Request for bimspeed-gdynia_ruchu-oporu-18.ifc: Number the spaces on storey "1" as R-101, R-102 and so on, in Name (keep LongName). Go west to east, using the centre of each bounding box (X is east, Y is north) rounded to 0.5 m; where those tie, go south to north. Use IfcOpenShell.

First a look at what the model holds.

```python
import ifcopenshell
import ifcopenshell.util.element
import ifcopenshell.util.placement

model = ifcopenshell.open("bimspeed-gdynia_ruchu-oporu-18.ifc")
print(model.schema)
storey = next(s for s in model.by_type("IfcBuildingStorey") if s.Name == "1")
spaces = [e for e in ifcopenshell.util.element.get_decomposition(storey) if e.is_a("IfcSpace")]
for e in sorted(spaces, key=lambda e: e.id()):
    origin = ifcopenshell.util.placement.get_local_placement(e.ObjectPlacement)[:3, 3]
    print(e.id(), e.Name, e.LongName, origin.round(2) + 0.0, sep=" | ")
```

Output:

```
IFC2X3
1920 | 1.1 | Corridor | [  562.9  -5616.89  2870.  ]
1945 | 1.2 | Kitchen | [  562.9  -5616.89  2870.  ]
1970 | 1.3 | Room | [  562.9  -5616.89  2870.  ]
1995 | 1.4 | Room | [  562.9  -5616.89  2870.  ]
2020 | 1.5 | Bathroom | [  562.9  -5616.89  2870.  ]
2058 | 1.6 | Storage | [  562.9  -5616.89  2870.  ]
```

```python
import ifcopenshell
import ifcopenshell.geom
import ifcopenshell.util.element
import ifcopenshell.util.shape

model = ifcopenshell.open("bimspeed-gdynia_ruchu-oporu-18.ifc")
settings = ifcopenshell.geom.settings()
settings.set("use-world-coords", True)


def centre(element):
    shape = ifcopenshell.geom.create_shape(settings, element)
    return ifcopenshell.util.shape.get_bbox_centroid(shape.geometry)


storey = next(s for s in model.by_type("IfcBuildingStorey") if s.Name == "1")
spaces = [e for e in ifcopenshell.util.element.get_decomposition(storey) if e.is_a("IfcSpace")]

# Insertion points can sit at a corner or the storey origin, so sort by the geometry (in metres).
centres = {e: centre(e) for e in spaces}
spaces.sort(key=lambda e: (round(centres[e][0] / 0.5), centres[e][1]))

for i, e in enumerate(spaces, start=1):
    number = f"R-1{i:02d}"
    e.Name = number
    print(e.id(), number)

model.write("bimspeed-gdynia_ruchu-oporu-18-out.ifc")
```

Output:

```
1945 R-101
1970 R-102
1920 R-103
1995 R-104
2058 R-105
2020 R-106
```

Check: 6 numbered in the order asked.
